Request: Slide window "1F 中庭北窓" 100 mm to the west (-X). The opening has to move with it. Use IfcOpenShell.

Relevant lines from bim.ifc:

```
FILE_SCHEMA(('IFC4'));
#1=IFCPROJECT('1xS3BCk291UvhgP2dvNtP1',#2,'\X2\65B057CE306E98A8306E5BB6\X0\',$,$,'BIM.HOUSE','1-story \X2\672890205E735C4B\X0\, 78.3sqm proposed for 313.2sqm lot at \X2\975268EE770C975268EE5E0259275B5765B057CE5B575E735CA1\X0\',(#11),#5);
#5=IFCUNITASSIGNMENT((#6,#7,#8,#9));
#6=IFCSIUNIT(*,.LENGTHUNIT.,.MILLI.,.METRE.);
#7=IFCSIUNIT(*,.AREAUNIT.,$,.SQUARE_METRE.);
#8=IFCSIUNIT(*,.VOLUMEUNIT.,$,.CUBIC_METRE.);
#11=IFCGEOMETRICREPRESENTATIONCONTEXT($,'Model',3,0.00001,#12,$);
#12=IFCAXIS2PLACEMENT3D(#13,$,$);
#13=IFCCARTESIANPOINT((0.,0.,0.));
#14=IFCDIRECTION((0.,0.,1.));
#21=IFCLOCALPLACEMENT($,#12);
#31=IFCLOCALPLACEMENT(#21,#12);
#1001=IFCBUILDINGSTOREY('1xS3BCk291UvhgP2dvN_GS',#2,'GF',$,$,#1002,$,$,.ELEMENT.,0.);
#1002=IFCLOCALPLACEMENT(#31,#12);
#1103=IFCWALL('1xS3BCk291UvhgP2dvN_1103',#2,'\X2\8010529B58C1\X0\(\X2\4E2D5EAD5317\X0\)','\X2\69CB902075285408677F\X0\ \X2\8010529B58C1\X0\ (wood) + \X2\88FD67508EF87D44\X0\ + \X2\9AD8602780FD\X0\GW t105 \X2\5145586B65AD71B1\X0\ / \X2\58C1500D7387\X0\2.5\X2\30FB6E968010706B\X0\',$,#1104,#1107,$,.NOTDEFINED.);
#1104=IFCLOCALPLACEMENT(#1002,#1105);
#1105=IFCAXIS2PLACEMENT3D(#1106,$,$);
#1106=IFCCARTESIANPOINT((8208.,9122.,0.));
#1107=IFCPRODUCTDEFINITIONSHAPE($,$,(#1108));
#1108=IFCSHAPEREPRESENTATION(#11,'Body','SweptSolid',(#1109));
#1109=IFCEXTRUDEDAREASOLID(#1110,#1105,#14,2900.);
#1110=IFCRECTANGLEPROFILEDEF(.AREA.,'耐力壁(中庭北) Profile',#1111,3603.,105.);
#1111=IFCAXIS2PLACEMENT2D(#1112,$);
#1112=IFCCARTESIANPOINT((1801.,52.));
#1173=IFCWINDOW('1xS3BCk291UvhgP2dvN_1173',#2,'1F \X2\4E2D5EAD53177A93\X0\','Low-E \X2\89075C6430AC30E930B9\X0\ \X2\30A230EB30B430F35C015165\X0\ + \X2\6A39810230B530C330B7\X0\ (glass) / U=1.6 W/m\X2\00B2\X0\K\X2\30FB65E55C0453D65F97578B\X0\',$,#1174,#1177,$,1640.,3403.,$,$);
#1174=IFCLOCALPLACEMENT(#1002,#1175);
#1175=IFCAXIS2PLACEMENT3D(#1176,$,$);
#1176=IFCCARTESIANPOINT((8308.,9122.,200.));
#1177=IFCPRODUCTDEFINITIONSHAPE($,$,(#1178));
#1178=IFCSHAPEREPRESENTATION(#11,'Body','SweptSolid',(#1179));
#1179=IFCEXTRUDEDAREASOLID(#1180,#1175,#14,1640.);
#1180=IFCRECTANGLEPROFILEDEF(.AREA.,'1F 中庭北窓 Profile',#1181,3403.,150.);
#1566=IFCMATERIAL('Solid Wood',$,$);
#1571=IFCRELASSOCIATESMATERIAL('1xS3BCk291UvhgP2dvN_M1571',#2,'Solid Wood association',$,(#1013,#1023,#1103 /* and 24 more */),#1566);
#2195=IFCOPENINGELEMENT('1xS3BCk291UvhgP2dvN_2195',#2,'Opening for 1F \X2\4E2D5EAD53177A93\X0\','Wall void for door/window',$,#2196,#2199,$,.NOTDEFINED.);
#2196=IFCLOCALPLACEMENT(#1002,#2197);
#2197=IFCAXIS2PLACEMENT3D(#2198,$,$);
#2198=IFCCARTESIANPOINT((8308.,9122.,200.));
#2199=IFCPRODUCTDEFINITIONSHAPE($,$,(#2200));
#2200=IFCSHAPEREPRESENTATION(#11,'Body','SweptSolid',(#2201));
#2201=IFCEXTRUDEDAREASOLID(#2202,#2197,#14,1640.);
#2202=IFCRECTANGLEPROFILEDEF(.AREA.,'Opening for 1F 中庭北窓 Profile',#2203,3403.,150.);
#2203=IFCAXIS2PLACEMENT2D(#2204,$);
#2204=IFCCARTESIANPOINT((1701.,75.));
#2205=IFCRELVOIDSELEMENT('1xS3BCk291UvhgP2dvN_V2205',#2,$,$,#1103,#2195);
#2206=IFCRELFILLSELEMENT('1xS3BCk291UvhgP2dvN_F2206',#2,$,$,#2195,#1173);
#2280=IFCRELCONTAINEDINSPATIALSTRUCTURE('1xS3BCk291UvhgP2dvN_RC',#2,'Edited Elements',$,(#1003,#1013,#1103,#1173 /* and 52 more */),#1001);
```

```python
import ifcopenshell
import ifcopenshell.api.geometry
import ifcopenshell.util.placement
import ifcopenshell.util.unit

model = ifcopenshell.open("bim.ifc")
unit_scale = ifcopenshell.util.unit.calculate_unit_scale(model)

window = model.by_guid("1xS3BCk291UvhgP2dvN_1173")
opening = window.FillsVoids[0].RelatingOpeningElement
wall = opening.VoidsElements[0].RelatingBuildingElement

wall_matrix = ifcopenshell.util.placement.get_local_placement(wall.ObjectPlacement)
shift = wall_matrix[:3, 0] * -0.1 / unit_scale
before = ifcopenshell.util.placement.get_local_placement(window.ObjectPlacement)[:3, 3].copy()

# The window is not placed relative to its opening, so move both.
for product in (opening, window):
    matrix = ifcopenshell.util.placement.get_local_placement(product.ObjectPlacement)
    matrix[:3, 3] += shift
    ifcopenshell.api.geometry.edit_object_placement(model, product=product, matrix=matrix, is_si=False)

after = ifcopenshell.util.placement.get_local_placement(window.ObjectPlacement)[:3, 3]
print("window moved by", (after - before).round(3) + 0.0)

model.write("bim-out.ifc")
```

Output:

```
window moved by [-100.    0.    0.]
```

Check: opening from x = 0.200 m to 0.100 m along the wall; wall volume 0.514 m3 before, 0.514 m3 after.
